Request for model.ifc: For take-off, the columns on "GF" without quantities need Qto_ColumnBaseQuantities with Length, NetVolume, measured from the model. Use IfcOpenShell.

First a look at what the model holds.

```python
import ifcopenshell
import ifcopenshell.util.element
import ifcopenshell.util.unit

model = ifcopenshell.open("model.ifc")
print(model.schema)
for unit_type in ("LENGTHUNIT", "AREAUNIT", "VOLUMEUNIT"):
    print(unit_type, ifcopenshell.util.unit.calculate_unit_scale(model, unit_type))
storey = next(s for s in model.by_type("IfcBuildingStorey") if s.Name == "GF")
columns = [e for e in ifcopenshell.util.element.get_decomposition(storey) if e.is_a("IfcColumn")]
for e in sorted(columns, key=lambda e: e.id()):
    print(e.id(), e.is_a(), e.Name, list(ifcopenshell.util.element.get_psets(e, qtos_only=True)), sep=" | ")
```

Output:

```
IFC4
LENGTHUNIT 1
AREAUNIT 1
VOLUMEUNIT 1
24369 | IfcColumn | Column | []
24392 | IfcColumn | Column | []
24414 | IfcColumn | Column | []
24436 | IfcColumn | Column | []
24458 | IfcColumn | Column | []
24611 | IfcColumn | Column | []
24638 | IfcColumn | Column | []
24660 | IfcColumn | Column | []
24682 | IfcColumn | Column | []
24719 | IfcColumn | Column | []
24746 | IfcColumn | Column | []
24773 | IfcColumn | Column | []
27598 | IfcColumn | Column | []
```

```python
import ifcopenshell
import ifcopenshell.api.pset
import ifcopenshell.geom
import ifcopenshell.util.element
import ifcopenshell.util.shape
import ifcopenshell.util.unit

model = ifcopenshell.open("model.ifc")
unit_scale = ifcopenshell.util.unit.calculate_unit_scale(model)
volume_scale = ifcopenshell.util.unit.calculate_unit_scale(model, "VOLUMEUNIT")
settings = ifcopenshell.geom.settings()

storey = next(s for s in model.by_type("IfcBuildingStorey") if s.Name == "GF")
columns = [e for e in ifcopenshell.util.element.get_decomposition(storey) if e.is_a("IfcColumn")]

for e in sorted(columns, key=lambda e: e.id()):
    if ifcopenshell.util.element.get_psets(e, qtos_only=True, should_inherit=False):
        continue
    # Geometry comes back in metres, in the element's own axes.
    shape = ifcopenshell.geom.create_shape(settings, e)
    values = {
        "Length": ifcopenshell.util.shape.get_z(shape.geometry) / unit_scale,
        "NetVolume": ifcopenshell.util.shape.get_volume(shape.geometry) / volume_scale,
    }
    qto = ifcopenshell.api.pset.add_qto(model, product=e, name="Qto_ColumnBaseQuantities")
    ifcopenshell.api.pset.edit_qto(model, qto=qto, properties=values)
    print(e.id(), {k: round(v, 3) for k, v in values.items()})

model.write("model_rev.ifc")
```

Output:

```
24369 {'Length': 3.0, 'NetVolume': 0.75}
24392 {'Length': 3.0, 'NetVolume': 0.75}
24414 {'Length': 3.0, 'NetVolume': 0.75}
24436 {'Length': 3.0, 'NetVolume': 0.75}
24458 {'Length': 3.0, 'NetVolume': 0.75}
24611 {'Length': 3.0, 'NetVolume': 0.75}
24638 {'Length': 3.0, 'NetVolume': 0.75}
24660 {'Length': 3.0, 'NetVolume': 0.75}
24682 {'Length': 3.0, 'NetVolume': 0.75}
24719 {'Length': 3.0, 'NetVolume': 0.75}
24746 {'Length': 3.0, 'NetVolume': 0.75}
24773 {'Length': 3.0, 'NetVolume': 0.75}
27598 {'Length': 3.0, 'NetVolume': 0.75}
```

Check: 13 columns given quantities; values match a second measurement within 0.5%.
